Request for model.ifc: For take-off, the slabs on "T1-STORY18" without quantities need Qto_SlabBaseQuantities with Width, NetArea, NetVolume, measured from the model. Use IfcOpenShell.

First a look at what the model holds.

```python
import ifcopenshell
import ifcopenshell.util.element
import ifcopenshell.util.unit

model = ifcopenshell.open("model.ifc")
print(model.schema)
for unit_type in ("LENGTHUNIT", "AREAUNIT", "VOLUMEUNIT"):
    print(unit_type, ifcopenshell.util.unit.calculate_unit_scale(model, unit_type))
storey = next(s for s in model.by_type("IfcBuildingStorey") if s.Name == "T1-STORY18")
slabs = [e for e in ifcopenshell.util.element.get_decomposition(storey) if e.is_a("IfcSlab")]
for e in sorted(slabs, key=lambda e: e.id()):
    print(e.id(), e.is_a(), e.Name, list(ifcopenshell.util.element.get_psets(e, qtos_only=True)), sep=" | ")
```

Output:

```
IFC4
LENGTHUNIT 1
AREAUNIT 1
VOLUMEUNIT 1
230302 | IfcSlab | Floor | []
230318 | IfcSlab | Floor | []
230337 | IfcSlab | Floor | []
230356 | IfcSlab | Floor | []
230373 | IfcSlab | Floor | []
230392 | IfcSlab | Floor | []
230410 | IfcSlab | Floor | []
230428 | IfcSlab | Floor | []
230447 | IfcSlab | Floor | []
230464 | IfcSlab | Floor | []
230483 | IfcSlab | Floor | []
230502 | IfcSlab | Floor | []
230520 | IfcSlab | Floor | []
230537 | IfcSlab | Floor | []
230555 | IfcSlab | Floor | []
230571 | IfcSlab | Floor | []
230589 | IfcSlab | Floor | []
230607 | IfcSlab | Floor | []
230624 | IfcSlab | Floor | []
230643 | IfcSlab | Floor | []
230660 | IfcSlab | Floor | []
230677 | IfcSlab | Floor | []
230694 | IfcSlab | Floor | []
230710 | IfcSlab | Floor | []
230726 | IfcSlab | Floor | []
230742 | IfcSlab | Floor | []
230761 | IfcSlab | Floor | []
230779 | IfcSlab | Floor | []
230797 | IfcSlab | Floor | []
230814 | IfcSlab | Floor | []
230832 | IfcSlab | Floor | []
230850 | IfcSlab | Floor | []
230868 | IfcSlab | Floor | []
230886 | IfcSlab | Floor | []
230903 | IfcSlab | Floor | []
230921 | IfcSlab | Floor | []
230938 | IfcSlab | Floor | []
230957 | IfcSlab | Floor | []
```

```python
import ifcopenshell
import ifcopenshell.api.pset
import ifcopenshell.geom
import ifcopenshell.util.element
import ifcopenshell.util.shape
import ifcopenshell.util.unit

model = ifcopenshell.open("model.ifc")
unit_scale = ifcopenshell.util.unit.calculate_unit_scale(model)
area_scale = ifcopenshell.util.unit.calculate_unit_scale(model, "AREAUNIT")
volume_scale = ifcopenshell.util.unit.calculate_unit_scale(model, "VOLUMEUNIT")
settings = ifcopenshell.geom.settings()

storey = next(s for s in model.by_type("IfcBuildingStorey") if s.Name == "T1-STORY18")
slabs = [e for e in ifcopenshell.util.element.get_decomposition(storey) if e.is_a("IfcSlab")]

for e in sorted(slabs, key=lambda e: e.id()):
    if ifcopenshell.util.element.get_psets(e, qtos_only=True, should_inherit=False):
        continue
    # Geometry comes back in metres, in the element's own axes.
    shape = ifcopenshell.geom.create_shape(settings, e)
    values = {
        "Width": ifcopenshell.util.shape.get_z(shape.geometry) / unit_scale,
        "NetArea": ifcopenshell.util.shape.get_footprint_area(shape.geometry) / area_scale,
        "NetVolume": ifcopenshell.util.shape.get_volume(shape.geometry) / volume_scale,
    }
    qto = ifcopenshell.api.pset.add_qto(model, product=e, name="Qto_SlabBaseQuantities")
    ifcopenshell.api.pset.edit_qto(model, qto=qto, properties=values)
    print(e.id(), {k: round(v, 3) for k, v in values.items()})

model.write("model_updated.ifc")
```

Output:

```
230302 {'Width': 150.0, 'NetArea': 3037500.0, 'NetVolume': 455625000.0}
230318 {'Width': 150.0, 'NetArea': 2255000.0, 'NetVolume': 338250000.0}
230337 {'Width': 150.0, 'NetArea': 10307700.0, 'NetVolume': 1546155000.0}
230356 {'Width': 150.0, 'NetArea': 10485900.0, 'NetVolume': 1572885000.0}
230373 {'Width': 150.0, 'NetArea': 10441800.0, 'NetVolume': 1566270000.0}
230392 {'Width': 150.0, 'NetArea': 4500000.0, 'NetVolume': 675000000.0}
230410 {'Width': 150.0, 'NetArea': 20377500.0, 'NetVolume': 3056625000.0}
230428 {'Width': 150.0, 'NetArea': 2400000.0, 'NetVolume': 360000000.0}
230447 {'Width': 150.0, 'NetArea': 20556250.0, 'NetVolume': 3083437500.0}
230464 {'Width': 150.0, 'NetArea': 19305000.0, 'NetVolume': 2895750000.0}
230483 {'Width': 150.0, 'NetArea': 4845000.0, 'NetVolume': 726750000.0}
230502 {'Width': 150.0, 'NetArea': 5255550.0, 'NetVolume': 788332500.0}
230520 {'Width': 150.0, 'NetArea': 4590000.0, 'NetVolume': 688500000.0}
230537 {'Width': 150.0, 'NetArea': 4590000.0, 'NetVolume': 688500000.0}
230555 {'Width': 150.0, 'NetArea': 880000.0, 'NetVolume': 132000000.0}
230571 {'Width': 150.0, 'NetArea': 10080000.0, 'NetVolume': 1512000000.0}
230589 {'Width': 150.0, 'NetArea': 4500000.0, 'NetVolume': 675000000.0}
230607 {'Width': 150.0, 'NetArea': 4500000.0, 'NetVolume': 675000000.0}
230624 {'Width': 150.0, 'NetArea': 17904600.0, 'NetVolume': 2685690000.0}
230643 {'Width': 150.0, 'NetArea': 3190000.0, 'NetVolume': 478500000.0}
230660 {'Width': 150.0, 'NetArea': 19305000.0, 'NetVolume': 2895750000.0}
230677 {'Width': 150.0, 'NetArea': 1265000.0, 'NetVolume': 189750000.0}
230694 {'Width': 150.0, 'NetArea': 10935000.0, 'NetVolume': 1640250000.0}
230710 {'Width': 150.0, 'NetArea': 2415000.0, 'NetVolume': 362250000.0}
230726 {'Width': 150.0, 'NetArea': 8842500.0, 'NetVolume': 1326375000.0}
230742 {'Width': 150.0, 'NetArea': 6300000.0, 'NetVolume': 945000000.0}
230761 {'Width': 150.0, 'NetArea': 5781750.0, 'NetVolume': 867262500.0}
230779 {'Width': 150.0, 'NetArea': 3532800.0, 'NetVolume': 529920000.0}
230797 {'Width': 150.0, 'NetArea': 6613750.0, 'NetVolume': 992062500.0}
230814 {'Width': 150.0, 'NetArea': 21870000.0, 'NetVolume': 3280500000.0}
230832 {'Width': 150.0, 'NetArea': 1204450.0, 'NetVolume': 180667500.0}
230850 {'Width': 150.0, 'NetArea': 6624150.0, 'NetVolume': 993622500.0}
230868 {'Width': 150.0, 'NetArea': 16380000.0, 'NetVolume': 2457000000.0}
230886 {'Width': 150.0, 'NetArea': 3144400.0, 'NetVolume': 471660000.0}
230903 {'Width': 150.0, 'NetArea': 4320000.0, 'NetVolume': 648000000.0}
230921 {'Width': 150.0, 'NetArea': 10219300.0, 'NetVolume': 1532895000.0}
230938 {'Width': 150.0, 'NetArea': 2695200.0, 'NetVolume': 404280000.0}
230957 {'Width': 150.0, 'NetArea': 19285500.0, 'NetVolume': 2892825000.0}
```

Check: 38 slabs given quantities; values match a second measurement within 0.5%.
